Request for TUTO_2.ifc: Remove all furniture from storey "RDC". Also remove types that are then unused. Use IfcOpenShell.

First a look at what the model holds.

```python
import ifcopenshell
import ifcopenshell.util.element

model = ifcopenshell.open("TUTO_2.ifc")
print(model.schema)
storey = next(s for s in model.by_type("IfcBuildingStorey") if s.Name == "RDC")
furniture = [e for e in ifcopenshell.util.element.get_decomposition(storey) if e.is_a("IfcFurnishingElement")]
seen = {}
for e in furniture:
    element_type = ifcopenshell.util.element.get_type(e)
    name = element_type.Name if element_type not in (None, e) else None
    seen[name] = seen.get(name, 0) + 1
for name, count in sorted(seen.items(), key=str):
    print(count, "x", name)
```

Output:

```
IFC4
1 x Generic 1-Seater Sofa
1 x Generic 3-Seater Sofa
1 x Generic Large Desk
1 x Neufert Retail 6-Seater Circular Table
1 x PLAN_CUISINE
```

```python
import ifcopenshell
import ifcopenshell.api.root
import ifcopenshell.util.element

model = ifcopenshell.open("TUTO_2.ifc")

storey = next(s for s in model.by_type("IfcBuildingStorey") if s.Name == "RDC")
furniture = [e for e in ifcopenshell.util.element.get_decomposition(storey) if e.is_a("IfcFurnishingElement")]
types = {ifcopenshell.util.element.get_type(e) for e in furniture} - {None, *furniture}

for e in furniture:
    ifcopenshell.api.root.remove_product(model, product=e)
print(len(furniture), "removed")

unused = [t for t in types if not ifcopenshell.util.element.get_types(t)]
for t in unused:
    ifcopenshell.api.root.remove_product(model, product=t)
print(len(unused), "unused types removed")

model.write("TUTO_2-out.ifc")
```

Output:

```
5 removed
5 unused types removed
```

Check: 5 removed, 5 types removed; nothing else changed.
